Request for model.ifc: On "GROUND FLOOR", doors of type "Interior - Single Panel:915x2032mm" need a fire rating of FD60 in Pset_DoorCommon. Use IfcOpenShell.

First a look at what the model holds.

```python
import ifcopenshell
import ifcopenshell.util.element

model = ifcopenshell.open("model.ifc")
print(model.schema)
storey = next(s for s in model.by_type("IfcBuildingStorey") if s.Name == "GROUND FLOOR")
doors = [e for e in ifcopenshell.util.element.get_decomposition(storey) if e.is_a("IfcDoor")]
seen = {}
for e in doors:
    element_type = ifcopenshell.util.element.get_type(e)
    key = (element_type.Name if element_type != e and element_type else None, ifcopenshell.util.element.get_pset(e, "Pset_DoorCommon", "FireRating"))
    seen[key] = seen.get(key, 0) + 1
for (name, value), count in sorted(seen.items(), key=str):
    print(count, "x", name, "|", value)
```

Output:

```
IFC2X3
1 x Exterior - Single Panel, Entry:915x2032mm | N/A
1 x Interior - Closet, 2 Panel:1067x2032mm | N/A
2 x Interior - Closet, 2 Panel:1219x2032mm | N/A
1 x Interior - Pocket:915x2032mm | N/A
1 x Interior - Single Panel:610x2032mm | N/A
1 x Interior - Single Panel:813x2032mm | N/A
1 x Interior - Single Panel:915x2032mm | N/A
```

```python
import ifcopenshell
import ifcopenshell.api.pset
import ifcopenshell.util.element

model = ifcopenshell.open("model.ifc")

storey = next(s for s in model.by_type("IfcBuildingStorey") if s.Name == "GROUND FLOOR")
doors = [e for e in ifcopenshell.util.element.get_decomposition(storey) if e.is_a("IfcDoor")]

count = 0
for e in doors:
    element_type = ifcopenshell.util.element.get_type(e)
    if element_type in (None, e) or element_type.Name != "Interior - Single Panel:915x2032mm":
        continue
    # add_pset returns the element's existing set when there is one.
    pset = ifcopenshell.api.pset.add_pset(model, product=e, name="Pset_DoorCommon")
    ifcopenshell.api.pset.edit_pset(model, pset=pset, properties={"FireRating": "FD60"})
    count += 1

print(count, "doors updated")

model.write("model_v2.ifc")
```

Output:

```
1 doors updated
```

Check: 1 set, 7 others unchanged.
